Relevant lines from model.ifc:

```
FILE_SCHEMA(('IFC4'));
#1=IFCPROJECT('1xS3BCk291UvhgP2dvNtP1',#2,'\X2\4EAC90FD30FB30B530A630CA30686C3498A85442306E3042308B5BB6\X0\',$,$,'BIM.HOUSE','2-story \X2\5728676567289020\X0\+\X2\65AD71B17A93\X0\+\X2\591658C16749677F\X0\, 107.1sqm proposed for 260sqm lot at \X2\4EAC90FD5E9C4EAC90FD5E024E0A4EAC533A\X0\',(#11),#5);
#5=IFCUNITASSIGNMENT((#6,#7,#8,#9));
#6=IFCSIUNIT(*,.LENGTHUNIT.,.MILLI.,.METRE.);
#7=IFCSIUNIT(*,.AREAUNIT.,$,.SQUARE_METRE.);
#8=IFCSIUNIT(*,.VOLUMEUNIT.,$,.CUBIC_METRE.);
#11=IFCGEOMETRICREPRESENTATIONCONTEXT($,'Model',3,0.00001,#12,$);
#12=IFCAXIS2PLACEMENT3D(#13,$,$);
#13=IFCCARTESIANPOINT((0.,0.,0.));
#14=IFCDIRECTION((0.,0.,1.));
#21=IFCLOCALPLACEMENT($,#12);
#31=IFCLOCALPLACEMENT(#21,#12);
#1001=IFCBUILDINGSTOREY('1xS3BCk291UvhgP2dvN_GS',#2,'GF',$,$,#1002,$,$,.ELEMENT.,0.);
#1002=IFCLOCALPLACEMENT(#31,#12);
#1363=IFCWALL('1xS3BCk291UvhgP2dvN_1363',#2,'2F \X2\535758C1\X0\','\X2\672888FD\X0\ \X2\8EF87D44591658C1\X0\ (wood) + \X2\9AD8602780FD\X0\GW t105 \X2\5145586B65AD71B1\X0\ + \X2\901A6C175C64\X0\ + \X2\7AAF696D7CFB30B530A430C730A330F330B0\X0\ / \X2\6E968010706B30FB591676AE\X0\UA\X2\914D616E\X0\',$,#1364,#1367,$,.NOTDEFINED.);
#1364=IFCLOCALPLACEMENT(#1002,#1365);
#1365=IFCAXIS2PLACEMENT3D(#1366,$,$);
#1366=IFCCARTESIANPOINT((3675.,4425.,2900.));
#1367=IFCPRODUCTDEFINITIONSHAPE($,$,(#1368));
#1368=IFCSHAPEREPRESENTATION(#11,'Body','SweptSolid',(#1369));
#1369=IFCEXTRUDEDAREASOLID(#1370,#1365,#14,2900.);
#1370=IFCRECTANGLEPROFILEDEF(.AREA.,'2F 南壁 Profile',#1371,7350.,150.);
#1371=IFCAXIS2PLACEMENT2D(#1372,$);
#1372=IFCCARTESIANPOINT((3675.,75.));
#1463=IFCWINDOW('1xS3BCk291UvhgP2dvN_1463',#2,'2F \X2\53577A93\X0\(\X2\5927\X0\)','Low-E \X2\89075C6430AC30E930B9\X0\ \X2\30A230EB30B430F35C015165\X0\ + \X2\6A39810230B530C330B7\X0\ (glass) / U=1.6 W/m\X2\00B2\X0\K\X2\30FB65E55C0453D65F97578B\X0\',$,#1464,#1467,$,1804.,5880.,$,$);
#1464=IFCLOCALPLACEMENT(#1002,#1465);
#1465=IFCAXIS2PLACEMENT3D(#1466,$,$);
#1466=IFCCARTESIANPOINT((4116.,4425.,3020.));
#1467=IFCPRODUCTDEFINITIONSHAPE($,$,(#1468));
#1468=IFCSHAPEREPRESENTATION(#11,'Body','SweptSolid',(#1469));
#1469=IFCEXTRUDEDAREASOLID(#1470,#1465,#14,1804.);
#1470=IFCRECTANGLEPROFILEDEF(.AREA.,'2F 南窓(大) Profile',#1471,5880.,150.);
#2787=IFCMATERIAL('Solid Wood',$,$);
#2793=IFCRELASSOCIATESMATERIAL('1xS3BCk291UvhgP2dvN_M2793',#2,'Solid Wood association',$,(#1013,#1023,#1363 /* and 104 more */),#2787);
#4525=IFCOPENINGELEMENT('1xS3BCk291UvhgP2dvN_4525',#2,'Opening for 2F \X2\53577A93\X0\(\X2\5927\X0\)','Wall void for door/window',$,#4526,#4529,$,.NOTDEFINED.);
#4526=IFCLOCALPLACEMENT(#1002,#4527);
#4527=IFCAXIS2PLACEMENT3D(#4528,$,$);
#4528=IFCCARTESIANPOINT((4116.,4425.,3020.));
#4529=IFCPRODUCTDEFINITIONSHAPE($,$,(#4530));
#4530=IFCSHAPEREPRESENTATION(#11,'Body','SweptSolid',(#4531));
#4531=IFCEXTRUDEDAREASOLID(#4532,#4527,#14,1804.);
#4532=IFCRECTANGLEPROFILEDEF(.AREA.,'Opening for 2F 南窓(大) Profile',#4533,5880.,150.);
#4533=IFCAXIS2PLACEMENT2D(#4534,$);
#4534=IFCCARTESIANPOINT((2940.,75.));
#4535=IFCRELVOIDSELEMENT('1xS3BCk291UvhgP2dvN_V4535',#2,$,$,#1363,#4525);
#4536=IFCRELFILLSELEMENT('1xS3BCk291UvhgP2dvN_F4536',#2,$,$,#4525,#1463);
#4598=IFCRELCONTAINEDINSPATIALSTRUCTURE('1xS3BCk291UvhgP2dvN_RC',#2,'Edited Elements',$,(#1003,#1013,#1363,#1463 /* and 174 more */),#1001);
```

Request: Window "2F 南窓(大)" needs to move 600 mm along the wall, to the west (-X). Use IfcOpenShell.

```python
import ifcopenshell
import ifcopenshell.api.geometry
import ifcopenshell.util.placement
import ifcopenshell.util.unit

model = ifcopenshell.open("model.ifc")
unit_scale = ifcopenshell.util.unit.calculate_unit_scale(model)

window = model.by_guid("1xS3BCk291UvhgP2dvN_1463")
opening = window.FillsVoids[0].RelatingOpeningElement
wall = opening.VoidsElements[0].RelatingBuildingElement

wall_matrix = ifcopenshell.util.placement.get_local_placement(wall.ObjectPlacement)
shift = wall_matrix[:3, 0] * -0.6 / unit_scale
before = ifcopenshell.util.placement.get_local_placement(window.ObjectPlacement)[:3, 3].copy()

# The window is not placed relative to its opening, so move both.
for product in (opening, window):
    matrix = ifcopenshell.util.placement.get_local_placement(product.ObjectPlacement)
    matrix[:3, 3] += shift
    ifcopenshell.api.geometry.edit_object_placement(model, product=product, matrix=matrix, is_si=False)

after = ifcopenshell.util.placement.get_local_placement(window.ObjectPlacement)[:3, 3]
print("window moved by", (after - before).round(3) + 0.0)

model.write("model_updated.ifc")
```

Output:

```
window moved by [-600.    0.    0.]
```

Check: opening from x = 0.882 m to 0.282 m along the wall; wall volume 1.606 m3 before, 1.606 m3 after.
